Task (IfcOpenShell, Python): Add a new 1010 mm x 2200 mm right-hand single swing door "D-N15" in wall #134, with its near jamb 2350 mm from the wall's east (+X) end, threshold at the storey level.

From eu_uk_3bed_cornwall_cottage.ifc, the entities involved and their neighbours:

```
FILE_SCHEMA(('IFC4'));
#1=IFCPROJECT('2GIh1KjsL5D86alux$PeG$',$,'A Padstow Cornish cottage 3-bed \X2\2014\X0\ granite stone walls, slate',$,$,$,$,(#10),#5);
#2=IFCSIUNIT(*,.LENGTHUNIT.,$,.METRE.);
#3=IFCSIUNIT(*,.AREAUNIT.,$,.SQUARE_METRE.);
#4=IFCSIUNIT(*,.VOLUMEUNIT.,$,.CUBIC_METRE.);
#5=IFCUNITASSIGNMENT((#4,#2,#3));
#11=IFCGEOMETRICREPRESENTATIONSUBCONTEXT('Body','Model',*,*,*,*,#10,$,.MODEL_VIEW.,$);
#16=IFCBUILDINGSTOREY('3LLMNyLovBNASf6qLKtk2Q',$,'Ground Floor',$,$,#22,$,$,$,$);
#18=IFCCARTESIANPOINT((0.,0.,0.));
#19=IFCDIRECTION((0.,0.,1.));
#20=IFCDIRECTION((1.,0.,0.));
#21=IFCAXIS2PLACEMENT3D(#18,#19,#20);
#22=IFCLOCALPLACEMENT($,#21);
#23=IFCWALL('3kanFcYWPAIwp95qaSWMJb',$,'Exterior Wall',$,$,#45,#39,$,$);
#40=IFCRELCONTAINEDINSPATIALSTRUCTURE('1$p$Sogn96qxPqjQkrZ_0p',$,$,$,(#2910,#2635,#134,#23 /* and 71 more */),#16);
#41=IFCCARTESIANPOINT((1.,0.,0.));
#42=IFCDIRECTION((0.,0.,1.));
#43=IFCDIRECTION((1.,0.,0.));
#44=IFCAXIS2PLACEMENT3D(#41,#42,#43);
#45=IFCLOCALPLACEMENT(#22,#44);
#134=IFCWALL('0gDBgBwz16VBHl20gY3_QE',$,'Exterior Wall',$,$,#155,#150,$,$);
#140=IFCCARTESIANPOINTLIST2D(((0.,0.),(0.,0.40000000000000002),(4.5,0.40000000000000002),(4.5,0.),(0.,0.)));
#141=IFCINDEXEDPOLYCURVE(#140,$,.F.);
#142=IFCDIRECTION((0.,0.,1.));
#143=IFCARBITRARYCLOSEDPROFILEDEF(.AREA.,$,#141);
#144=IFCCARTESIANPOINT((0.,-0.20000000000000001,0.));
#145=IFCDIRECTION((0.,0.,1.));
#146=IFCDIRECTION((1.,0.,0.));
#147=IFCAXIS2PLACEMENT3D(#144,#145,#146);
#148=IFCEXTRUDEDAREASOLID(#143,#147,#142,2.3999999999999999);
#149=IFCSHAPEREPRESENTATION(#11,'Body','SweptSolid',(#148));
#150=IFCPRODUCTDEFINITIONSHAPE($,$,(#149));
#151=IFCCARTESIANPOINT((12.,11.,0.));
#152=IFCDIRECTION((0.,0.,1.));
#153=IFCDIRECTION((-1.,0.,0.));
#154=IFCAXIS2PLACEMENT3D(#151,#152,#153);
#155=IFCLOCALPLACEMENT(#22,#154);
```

```python
import numpy as np
import ifcopenshell
import ifcopenshell.api.feature
import ifcopenshell.api.geometry
import ifcopenshell.api.root
import ifcopenshell.api.spatial
import ifcopenshell.geom
import ifcopenshell.util.element
import ifcopenshell.util.placement
import ifcopenshell.util.representation
import ifcopenshell.util.shape
import ifcopenshell.util.unit

model = ifcopenshell.open("eu_uk_3bed_cornwall_cottage.ifc")
unit_scale = ifcopenshell.util.unit.calculate_unit_scale(model)
settings = ifcopenshell.geom.settings()


def volume(element):
    """Net volume in cubic metres, openings subtracted."""
    shape = ifcopenshell.geom.create_shape(settings, element)
    return ifcopenshell.util.shape.get_volume(shape.geometry)


wall = model.by_guid("0gDBgBwz16VBHl20gY3_QE")
storey = ifcopenshell.util.element.get_container(wall, ifc_class="IfcBuildingStorey")
context = ifcopenshell.util.representation.get_context(model, "Model", "Body", "MODEL_VIEW")
before = volume(wall)

width, height, from_end, sill = 1.01, 2.2, 2.35, 0.0  # metres

# The wall runs along its own X axis, and the end named is its -X end.
wall_shape = ifcopenshell.geom.create_shape(settings, wall)
x, y, z = ifcopenshell.util.shape.get_vertices(wall_shape.geometry).T
start = x.min() + from_end
face, thickness = float(y.min()), float(y.max() - y.min())
wall_matrix = ifcopenshell.util.placement.get_local_placement(wall.ObjectPlacement)
level = ifcopenshell.util.placement.get_local_placement(storey.ObjectPlacement)[2, 3]


def in_wall(x, y):
    """Placement at x, y metres in the wall's axes, at sill height."""
    matrix = wall_matrix.copy()
    matrix[:, 3] = wall_matrix @ np.array([x / unit_scale, y / unit_scale, 0.0, 1.0])
    matrix[2, 3] = level + sill / unit_scale
    return matrix


# Opening: a box that overshoots both wall faces by 50 mm.
opening = ifcopenshell.api.root.create_entity(model, ifc_class="IfcOpeningElement", predefined_type="OPENING")
box = ifcopenshell.api.geometry.add_wall_representation(
    model, context=context, length=width, height=height, thickness=thickness + 0.1
)
ifcopenshell.api.geometry.assign_representation(model, product=opening, representation=box)
ifcopenshell.api.geometry.edit_object_placement(model, product=opening, matrix=in_wall(start, face - 0.05), is_si=False)
ifcopenshell.api.feature.add_feature(model, feature=opening, element=wall)

door = ifcopenshell.api.root.create_entity(model, ifc_class="IfcDoor", name="D-N15", predefined_type="DOOR")
door.OverallWidth, door.OverallHeight = width / unit_scale, height / unit_scale
door.OperationType = "SINGLE_SWING_RIGHT"
body = ifcopenshell.api.geometry.add_door_representation(
    model,
    context=context,
    overall_width=door.OverallWidth,
    overall_height=door.OverallHeight,
    operation_type="SINGLE_SWING_RIGHT",
    lining_properties={"LiningDepth": thickness / unit_scale, "ThresholdDepth": thickness / unit_scale},
)
ifcopenshell.api.geometry.assign_representation(model, product=door, representation=body)
ifcopenshell.api.spatial.assign_container(model, products=[door], relating_structure=storey)
ifcopenshell.api.feature.add_filling(model, opening=opening, element=door)

# The lining spans the wall, so the door starts at the wall face.
ifcopenshell.api.geometry.edit_object_placement(model, product=door, matrix=in_wall(start, face), is_si=False)

after = volume(wall)

print(f"wall volume {before:.3f} -> {after:.3f} m3")

model.write("eu_uk_3bed_cornwall_cottage_updated.ifc")
```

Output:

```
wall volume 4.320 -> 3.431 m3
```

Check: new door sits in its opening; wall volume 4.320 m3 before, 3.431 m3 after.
